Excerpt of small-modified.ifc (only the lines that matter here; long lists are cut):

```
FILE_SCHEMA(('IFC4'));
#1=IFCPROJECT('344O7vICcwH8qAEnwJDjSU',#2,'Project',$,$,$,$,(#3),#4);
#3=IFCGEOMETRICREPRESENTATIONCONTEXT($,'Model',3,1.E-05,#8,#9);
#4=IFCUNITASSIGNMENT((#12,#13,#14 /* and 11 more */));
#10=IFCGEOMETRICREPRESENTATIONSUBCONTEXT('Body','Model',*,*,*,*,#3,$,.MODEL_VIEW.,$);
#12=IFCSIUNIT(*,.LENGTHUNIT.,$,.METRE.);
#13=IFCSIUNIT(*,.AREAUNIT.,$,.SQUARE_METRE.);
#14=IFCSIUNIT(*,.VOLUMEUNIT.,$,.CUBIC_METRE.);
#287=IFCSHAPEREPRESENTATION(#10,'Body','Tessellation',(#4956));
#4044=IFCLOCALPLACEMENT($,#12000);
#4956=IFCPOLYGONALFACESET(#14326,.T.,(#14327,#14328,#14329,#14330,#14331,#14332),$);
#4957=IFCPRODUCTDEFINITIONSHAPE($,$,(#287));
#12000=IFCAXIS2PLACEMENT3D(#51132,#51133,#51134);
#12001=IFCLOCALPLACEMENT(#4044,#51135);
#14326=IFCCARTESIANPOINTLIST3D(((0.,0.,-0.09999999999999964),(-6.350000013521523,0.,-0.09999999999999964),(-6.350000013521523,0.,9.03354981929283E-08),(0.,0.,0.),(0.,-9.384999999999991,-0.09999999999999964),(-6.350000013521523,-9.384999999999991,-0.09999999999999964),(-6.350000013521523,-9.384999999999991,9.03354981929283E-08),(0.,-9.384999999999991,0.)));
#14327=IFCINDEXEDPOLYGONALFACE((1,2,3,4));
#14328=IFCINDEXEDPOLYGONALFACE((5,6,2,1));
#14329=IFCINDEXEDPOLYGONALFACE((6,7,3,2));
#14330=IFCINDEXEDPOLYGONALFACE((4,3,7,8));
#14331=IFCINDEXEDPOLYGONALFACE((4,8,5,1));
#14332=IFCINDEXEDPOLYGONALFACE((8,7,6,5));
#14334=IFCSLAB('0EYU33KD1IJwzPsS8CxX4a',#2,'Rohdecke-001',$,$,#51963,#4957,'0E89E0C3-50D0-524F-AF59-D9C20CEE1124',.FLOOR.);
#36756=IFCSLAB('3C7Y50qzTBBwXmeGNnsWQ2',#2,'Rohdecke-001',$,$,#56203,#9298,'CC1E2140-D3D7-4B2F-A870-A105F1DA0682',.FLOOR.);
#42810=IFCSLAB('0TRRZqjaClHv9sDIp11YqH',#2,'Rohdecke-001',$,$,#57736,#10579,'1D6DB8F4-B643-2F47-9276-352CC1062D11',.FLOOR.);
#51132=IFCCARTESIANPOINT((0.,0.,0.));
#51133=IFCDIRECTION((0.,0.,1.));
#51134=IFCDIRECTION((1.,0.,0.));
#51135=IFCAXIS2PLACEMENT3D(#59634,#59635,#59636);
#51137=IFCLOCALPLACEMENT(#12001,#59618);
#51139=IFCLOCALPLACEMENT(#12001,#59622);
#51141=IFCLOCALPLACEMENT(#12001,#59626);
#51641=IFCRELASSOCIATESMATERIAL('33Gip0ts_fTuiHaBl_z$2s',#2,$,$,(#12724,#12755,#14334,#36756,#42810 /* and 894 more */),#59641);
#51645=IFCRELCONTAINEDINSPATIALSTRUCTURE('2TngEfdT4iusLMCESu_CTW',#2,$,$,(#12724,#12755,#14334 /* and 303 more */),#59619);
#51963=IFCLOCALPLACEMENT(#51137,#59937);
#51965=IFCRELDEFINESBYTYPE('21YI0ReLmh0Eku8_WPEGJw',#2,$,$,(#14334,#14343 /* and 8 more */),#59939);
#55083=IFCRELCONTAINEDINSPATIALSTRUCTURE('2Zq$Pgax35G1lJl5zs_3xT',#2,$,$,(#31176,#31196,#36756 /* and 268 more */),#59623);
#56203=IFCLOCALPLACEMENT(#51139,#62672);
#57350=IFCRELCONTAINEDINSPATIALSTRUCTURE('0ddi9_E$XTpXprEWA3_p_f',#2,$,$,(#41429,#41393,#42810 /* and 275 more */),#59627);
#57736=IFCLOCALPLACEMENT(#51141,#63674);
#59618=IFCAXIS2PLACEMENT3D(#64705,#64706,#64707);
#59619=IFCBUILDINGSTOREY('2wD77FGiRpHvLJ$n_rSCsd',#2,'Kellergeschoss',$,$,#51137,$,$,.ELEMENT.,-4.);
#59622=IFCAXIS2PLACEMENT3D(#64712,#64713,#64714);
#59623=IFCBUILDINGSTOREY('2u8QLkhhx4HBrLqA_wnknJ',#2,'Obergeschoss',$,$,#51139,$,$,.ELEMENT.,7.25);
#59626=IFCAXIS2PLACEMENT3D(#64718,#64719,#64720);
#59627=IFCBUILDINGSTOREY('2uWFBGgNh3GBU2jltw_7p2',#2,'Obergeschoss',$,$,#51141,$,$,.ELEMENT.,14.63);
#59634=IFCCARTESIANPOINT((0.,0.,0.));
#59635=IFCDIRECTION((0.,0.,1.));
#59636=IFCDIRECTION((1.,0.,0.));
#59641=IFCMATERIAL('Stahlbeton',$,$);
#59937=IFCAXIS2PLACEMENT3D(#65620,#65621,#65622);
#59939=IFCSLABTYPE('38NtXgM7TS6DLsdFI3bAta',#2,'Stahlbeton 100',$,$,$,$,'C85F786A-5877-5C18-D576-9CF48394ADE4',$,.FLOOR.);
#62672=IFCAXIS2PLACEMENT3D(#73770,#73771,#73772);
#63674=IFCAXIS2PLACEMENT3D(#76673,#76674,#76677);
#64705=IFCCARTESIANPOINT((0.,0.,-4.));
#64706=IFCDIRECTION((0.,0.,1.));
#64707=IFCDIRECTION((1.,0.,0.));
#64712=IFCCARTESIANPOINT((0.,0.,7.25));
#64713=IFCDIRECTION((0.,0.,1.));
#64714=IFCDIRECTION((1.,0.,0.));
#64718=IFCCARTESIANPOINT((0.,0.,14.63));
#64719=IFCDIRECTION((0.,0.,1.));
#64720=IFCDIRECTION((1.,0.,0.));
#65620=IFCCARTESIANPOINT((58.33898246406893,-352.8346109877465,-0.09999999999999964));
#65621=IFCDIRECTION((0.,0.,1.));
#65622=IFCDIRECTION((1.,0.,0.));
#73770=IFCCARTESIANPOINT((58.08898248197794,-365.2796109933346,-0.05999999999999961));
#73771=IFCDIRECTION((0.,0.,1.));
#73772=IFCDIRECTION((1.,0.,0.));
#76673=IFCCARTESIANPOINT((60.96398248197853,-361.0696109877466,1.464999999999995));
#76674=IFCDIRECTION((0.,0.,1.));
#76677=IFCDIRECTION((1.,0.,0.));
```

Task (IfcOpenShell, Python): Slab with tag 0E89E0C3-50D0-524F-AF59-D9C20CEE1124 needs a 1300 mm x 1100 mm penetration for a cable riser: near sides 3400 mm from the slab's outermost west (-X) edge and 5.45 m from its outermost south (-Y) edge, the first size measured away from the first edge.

```python
import numpy as np
import ifcopenshell
import ifcopenshell.api.feature
import ifcopenshell.api.geometry
import ifcopenshell.api.root
import ifcopenshell.geom
import ifcopenshell.util.placement
import ifcopenshell.util.representation
import ifcopenshell.util.shape
import ifcopenshell.util.unit

model = ifcopenshell.open("small-modified.ifc")
unit_scale = ifcopenshell.util.unit.calculate_unit_scale(model)
settings = ifcopenshell.geom.settings()


def volume(element):
    """Net volume in cubic metres, openings subtracted."""
    shape = ifcopenshell.geom.create_shape(settings, element)
    return ifcopenshell.util.shape.get_volume(shape.geometry)


slab = model.by_guid("0EYU33KD1IJwzPsS8CxX4a")
before = volume(slab)

# Extent in the slab's own axes, in metres. The edges named are its -X and -Y sides.
slab_shape = ifcopenshell.geom.create_shape(settings, slab)
vertices = ifcopenshell.util.shape.get_vertices(slab_shape.geometry)
x_min, y_min, bottom = vertices.min(axis=0)
top = vertices[:, 2].max()

opening = ifcopenshell.api.root.create_entity(model, ifc_class="IfcOpeningElement", name="Cable riser opening", predefined_type="OPENING")
context = ifcopenshell.util.representation.get_context(model, "Model", "Body", "MODEL_VIEW")
width, depth = 1.3, 1.1
outline = [(0.0, 0.0), (width, 0.0), (width, depth), (0.0, depth), (0.0, 0.0)]
# Overshoot both faces by 50 mm so the cut is clean.
shape = ifcopenshell.api.geometry.add_slab_representation(
    model, context=context, depth=top - bottom + 0.1, polyline=outline
)
ifcopenshell.api.geometry.assign_representation(model, product=opening, representation=shape)

matrix = ifcopenshell.util.placement.get_local_placement(slab.ObjectPlacement)
matrix[:, 3] = matrix @ np.append(np.array([x_min + 3.4, y_min + 5.45, bottom - 0.05]) / unit_scale, 1.0)
ifcopenshell.api.geometry.edit_object_placement(model, product=opening, matrix=matrix, is_si=False)
ifcopenshell.api.feature.add_feature(model, feature=opening, element=slab)

after = volume(slab)

print(f"slab volume {before:.3f} -> {after:.3f} m3")

model.write("small-modified_updated.ifc")
```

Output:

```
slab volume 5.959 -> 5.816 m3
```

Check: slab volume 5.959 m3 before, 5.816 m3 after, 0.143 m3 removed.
